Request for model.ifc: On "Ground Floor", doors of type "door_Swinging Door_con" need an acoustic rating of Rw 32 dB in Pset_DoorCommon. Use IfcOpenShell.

First a look at what the model holds.

```python
import ifcopenshell
import ifcopenshell.util.element

model = ifcopenshell.open("model.ifc")
print(model.schema)
storey = next(s for s in model.by_type("IfcBuildingStorey") if s.Name == "Ground Floor")
doors = [e for e in ifcopenshell.util.element.get_decomposition(storey) if e.is_a("IfcDoor")]
seen = {}
for e in doors:
    element_type = ifcopenshell.util.element.get_type(e)
    key = (element_type.Name if element_type != e and element_type else None, ifcopenshell.util.element.get_pset(e, "Pset_DoorCommon", "AcousticRating"))
    seen[key] = seen.get(key, 0) + 1
for (name, value), count in sorted(seen.items(), key=str):
    print(count, "x", name, "|", value)
```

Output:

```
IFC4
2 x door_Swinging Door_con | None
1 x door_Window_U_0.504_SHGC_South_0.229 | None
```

```python
import ifcopenshell
import ifcopenshell.api.pset
import ifcopenshell.util.element

model = ifcopenshell.open("model.ifc")

storey = next(s for s in model.by_type("IfcBuildingStorey") if s.Name == "Ground Floor")
doors = [e for e in ifcopenshell.util.element.get_decomposition(storey) if e.is_a("IfcDoor")]

count = 0
for e in doors:
    element_type = ifcopenshell.util.element.get_type(e)
    if element_type in (None, e) or element_type.Name != "door_Swinging Door_con":
        continue
    # add_pset returns the element's existing set when there is one.
    pset = ifcopenshell.api.pset.add_pset(model, product=e, name="Pset_DoorCommon")
    ifcopenshell.api.pset.edit_pset(model, pset=pset, properties={"AcousticRating": "Rw 32 dB"})
    count += 1

print(count, "doors updated")

model.write("model_v2.ifc")
```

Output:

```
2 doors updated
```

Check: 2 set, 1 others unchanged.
